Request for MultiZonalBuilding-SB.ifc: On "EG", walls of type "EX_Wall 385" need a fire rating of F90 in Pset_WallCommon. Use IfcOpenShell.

First a look at what the model holds.

```python
import ifcopenshell
import ifcopenshell.util.element

model = ifcopenshell.open("MultiZonalBuilding-SB.ifc")
print(model.schema)
storey = next(s for s in model.by_type("IfcBuildingStorey") if s.Name == "EG")
walls = [e for e in ifcopenshell.util.element.get_decomposition(storey) if e.is_a("IfcWall")]
seen = {}
for e in walls:
    element_type = ifcopenshell.util.element.get_type(e)
    key = (element_type.Name if element_type != e and element_type else None, ifcopenshell.util.element.get_pset(e, "Pset_WallCommon", "FireRating"))
    seen[key] = seen.get(key, 0) + 1
for (name, value), count in sorted(seen.items(), key=str):
    print(count, "x", name, "|", value)
```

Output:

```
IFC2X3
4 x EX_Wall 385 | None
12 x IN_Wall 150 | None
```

```python
import ifcopenshell
import ifcopenshell.api.pset
import ifcopenshell.util.element

model = ifcopenshell.open("MultiZonalBuilding-SB.ifc")

storey = next(s for s in model.by_type("IfcBuildingStorey") if s.Name == "EG")
walls = [e for e in ifcopenshell.util.element.get_decomposition(storey) if e.is_a("IfcWall")]

count = 0
for e in walls:
    element_type = ifcopenshell.util.element.get_type(e)
    if element_type in (None, e) or element_type.Name != "EX_Wall 385":
        continue
    # add_pset returns the element's existing set when there is one.
    pset = ifcopenshell.api.pset.add_pset(model, product=e, name="Pset_WallCommon")
    ifcopenshell.api.pset.edit_pset(model, pset=pset, properties={"FireRating": "F90"})
    count += 1

print(count, "walls updated")

model.write("MultiZonalBuilding-SB_edited.ifc")
```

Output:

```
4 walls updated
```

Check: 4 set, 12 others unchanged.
